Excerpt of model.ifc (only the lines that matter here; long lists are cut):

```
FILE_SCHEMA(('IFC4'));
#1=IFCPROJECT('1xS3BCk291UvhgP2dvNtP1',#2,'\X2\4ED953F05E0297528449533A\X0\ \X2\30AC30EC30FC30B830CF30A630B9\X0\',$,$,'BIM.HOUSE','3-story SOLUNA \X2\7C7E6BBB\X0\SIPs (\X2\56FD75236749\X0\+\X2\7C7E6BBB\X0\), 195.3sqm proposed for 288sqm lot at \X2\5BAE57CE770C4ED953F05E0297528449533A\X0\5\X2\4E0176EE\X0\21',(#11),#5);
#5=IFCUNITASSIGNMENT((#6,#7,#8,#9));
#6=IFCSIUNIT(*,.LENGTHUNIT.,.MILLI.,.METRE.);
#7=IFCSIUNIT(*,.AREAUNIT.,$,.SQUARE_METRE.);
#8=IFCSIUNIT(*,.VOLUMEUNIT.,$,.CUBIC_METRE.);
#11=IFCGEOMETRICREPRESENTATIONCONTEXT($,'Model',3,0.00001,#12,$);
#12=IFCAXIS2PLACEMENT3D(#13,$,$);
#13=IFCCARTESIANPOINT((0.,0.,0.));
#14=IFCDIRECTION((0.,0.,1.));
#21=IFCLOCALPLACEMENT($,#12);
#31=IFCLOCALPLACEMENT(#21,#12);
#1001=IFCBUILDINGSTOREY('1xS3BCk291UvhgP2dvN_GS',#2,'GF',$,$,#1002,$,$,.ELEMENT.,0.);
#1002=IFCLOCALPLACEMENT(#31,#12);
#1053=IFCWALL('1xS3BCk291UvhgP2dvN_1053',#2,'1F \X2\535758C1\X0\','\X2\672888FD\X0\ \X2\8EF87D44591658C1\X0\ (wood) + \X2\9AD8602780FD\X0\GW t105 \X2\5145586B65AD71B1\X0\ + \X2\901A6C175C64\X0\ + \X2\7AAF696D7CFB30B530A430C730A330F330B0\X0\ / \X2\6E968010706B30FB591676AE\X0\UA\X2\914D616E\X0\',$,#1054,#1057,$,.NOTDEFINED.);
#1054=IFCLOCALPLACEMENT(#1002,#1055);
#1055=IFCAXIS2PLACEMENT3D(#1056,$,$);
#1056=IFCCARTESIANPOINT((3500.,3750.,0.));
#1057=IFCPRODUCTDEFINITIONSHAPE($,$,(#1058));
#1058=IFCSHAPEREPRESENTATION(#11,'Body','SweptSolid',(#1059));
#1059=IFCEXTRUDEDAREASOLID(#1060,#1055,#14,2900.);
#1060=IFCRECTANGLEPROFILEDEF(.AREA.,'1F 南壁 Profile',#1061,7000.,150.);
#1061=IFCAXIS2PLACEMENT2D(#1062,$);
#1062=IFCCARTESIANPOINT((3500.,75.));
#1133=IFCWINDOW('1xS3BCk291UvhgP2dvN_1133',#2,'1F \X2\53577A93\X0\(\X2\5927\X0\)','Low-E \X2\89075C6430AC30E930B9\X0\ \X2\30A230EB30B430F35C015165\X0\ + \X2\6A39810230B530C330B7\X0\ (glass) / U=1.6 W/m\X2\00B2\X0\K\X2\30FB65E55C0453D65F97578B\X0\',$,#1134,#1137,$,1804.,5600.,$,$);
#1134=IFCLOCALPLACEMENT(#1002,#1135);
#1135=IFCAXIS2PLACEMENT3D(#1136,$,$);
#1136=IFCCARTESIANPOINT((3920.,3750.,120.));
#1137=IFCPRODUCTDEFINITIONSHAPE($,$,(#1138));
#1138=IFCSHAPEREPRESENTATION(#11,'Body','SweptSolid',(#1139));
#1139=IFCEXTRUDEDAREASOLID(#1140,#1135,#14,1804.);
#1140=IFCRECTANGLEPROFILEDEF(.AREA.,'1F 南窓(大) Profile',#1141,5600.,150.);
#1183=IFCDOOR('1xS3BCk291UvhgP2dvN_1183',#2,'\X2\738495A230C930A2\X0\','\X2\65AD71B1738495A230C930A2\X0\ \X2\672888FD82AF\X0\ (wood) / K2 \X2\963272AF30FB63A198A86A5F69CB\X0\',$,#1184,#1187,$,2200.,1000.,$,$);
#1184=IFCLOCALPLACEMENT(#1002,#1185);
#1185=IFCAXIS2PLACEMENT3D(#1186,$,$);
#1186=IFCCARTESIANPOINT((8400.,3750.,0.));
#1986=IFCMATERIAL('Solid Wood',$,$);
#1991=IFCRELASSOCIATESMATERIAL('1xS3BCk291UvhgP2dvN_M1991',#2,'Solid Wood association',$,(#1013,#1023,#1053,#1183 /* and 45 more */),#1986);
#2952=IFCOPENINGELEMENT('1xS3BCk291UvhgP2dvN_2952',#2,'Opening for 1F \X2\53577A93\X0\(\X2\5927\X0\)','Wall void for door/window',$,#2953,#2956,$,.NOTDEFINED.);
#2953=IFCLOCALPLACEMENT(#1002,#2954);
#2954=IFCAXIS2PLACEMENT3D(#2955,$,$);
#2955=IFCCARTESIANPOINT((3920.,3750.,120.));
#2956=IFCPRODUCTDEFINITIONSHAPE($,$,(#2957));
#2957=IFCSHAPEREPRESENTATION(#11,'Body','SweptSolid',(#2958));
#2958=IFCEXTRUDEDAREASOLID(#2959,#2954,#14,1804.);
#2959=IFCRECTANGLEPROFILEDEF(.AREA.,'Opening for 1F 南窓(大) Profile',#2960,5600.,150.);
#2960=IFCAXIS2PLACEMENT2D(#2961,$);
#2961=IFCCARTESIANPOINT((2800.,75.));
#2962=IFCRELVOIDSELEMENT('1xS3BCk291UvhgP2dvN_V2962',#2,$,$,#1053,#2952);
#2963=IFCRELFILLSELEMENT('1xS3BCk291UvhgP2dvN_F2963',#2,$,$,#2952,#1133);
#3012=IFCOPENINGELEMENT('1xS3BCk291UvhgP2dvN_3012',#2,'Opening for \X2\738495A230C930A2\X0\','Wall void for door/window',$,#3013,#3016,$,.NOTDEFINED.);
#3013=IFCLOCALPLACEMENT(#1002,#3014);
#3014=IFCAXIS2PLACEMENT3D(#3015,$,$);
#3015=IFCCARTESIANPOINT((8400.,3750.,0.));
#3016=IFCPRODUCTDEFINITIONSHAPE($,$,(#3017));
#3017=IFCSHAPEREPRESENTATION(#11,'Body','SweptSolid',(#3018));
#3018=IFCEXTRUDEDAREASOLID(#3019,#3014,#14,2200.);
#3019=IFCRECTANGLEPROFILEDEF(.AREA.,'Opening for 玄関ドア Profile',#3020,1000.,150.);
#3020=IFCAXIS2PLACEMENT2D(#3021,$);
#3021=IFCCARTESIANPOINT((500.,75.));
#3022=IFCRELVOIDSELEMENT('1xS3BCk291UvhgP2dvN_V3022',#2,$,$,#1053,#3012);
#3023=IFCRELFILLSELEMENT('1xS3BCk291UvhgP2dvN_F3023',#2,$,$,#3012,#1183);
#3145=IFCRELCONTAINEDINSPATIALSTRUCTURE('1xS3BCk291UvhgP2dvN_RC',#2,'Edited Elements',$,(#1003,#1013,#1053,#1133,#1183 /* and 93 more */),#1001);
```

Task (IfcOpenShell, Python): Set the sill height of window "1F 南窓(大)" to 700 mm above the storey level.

```python
import numpy as np
import ifcopenshell
import ifcopenshell.api.geometry
import ifcopenshell.geom
import ifcopenshell.util.element
import ifcopenshell.util.placement
import ifcopenshell.util.shape
import ifcopenshell.util.unit

model = ifcopenshell.open("model.ifc")
unit_scale = ifcopenshell.util.unit.calculate_unit_scale(model)

window = model.by_guid("1xS3BCk291UvhgP2dvN_1133")
opening = window.FillsVoids[0].RelatingOpeningElement
storey = ifcopenshell.util.element.get_container(window, ifc_class="IfcBuildingStorey")
level = ifcopenshell.util.placement.get_local_placement(storey.ObjectPlacement)[2, 3]

# The opening's origin need not be at the sill, so measure its lowest point.
shape = ifcopenshell.geom.create_shape(ifcopenshell.geom.settings(), opening)
bottom = ifcopenshell.util.shape.get_shape_bottom_elevation(shape, shape.geometry) / unit_scale
dz = level + 0.7 / unit_scale - bottom

shift = np.array([0.0, 0.0, dz])
# The window is not placed relative to its opening, so move both.
for product in (opening, window):
    matrix = ifcopenshell.util.placement.get_local_placement(product.ObjectPlacement)
    matrix[:3, 3] += shift
    ifcopenshell.api.geometry.edit_object_placement(model, product=product, matrix=matrix, is_si=False)

print(f"moved by {dz * unit_scale:+.3f} m")

model.write("model-out.ifc")
```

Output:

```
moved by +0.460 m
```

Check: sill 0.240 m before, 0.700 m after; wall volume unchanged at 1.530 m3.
